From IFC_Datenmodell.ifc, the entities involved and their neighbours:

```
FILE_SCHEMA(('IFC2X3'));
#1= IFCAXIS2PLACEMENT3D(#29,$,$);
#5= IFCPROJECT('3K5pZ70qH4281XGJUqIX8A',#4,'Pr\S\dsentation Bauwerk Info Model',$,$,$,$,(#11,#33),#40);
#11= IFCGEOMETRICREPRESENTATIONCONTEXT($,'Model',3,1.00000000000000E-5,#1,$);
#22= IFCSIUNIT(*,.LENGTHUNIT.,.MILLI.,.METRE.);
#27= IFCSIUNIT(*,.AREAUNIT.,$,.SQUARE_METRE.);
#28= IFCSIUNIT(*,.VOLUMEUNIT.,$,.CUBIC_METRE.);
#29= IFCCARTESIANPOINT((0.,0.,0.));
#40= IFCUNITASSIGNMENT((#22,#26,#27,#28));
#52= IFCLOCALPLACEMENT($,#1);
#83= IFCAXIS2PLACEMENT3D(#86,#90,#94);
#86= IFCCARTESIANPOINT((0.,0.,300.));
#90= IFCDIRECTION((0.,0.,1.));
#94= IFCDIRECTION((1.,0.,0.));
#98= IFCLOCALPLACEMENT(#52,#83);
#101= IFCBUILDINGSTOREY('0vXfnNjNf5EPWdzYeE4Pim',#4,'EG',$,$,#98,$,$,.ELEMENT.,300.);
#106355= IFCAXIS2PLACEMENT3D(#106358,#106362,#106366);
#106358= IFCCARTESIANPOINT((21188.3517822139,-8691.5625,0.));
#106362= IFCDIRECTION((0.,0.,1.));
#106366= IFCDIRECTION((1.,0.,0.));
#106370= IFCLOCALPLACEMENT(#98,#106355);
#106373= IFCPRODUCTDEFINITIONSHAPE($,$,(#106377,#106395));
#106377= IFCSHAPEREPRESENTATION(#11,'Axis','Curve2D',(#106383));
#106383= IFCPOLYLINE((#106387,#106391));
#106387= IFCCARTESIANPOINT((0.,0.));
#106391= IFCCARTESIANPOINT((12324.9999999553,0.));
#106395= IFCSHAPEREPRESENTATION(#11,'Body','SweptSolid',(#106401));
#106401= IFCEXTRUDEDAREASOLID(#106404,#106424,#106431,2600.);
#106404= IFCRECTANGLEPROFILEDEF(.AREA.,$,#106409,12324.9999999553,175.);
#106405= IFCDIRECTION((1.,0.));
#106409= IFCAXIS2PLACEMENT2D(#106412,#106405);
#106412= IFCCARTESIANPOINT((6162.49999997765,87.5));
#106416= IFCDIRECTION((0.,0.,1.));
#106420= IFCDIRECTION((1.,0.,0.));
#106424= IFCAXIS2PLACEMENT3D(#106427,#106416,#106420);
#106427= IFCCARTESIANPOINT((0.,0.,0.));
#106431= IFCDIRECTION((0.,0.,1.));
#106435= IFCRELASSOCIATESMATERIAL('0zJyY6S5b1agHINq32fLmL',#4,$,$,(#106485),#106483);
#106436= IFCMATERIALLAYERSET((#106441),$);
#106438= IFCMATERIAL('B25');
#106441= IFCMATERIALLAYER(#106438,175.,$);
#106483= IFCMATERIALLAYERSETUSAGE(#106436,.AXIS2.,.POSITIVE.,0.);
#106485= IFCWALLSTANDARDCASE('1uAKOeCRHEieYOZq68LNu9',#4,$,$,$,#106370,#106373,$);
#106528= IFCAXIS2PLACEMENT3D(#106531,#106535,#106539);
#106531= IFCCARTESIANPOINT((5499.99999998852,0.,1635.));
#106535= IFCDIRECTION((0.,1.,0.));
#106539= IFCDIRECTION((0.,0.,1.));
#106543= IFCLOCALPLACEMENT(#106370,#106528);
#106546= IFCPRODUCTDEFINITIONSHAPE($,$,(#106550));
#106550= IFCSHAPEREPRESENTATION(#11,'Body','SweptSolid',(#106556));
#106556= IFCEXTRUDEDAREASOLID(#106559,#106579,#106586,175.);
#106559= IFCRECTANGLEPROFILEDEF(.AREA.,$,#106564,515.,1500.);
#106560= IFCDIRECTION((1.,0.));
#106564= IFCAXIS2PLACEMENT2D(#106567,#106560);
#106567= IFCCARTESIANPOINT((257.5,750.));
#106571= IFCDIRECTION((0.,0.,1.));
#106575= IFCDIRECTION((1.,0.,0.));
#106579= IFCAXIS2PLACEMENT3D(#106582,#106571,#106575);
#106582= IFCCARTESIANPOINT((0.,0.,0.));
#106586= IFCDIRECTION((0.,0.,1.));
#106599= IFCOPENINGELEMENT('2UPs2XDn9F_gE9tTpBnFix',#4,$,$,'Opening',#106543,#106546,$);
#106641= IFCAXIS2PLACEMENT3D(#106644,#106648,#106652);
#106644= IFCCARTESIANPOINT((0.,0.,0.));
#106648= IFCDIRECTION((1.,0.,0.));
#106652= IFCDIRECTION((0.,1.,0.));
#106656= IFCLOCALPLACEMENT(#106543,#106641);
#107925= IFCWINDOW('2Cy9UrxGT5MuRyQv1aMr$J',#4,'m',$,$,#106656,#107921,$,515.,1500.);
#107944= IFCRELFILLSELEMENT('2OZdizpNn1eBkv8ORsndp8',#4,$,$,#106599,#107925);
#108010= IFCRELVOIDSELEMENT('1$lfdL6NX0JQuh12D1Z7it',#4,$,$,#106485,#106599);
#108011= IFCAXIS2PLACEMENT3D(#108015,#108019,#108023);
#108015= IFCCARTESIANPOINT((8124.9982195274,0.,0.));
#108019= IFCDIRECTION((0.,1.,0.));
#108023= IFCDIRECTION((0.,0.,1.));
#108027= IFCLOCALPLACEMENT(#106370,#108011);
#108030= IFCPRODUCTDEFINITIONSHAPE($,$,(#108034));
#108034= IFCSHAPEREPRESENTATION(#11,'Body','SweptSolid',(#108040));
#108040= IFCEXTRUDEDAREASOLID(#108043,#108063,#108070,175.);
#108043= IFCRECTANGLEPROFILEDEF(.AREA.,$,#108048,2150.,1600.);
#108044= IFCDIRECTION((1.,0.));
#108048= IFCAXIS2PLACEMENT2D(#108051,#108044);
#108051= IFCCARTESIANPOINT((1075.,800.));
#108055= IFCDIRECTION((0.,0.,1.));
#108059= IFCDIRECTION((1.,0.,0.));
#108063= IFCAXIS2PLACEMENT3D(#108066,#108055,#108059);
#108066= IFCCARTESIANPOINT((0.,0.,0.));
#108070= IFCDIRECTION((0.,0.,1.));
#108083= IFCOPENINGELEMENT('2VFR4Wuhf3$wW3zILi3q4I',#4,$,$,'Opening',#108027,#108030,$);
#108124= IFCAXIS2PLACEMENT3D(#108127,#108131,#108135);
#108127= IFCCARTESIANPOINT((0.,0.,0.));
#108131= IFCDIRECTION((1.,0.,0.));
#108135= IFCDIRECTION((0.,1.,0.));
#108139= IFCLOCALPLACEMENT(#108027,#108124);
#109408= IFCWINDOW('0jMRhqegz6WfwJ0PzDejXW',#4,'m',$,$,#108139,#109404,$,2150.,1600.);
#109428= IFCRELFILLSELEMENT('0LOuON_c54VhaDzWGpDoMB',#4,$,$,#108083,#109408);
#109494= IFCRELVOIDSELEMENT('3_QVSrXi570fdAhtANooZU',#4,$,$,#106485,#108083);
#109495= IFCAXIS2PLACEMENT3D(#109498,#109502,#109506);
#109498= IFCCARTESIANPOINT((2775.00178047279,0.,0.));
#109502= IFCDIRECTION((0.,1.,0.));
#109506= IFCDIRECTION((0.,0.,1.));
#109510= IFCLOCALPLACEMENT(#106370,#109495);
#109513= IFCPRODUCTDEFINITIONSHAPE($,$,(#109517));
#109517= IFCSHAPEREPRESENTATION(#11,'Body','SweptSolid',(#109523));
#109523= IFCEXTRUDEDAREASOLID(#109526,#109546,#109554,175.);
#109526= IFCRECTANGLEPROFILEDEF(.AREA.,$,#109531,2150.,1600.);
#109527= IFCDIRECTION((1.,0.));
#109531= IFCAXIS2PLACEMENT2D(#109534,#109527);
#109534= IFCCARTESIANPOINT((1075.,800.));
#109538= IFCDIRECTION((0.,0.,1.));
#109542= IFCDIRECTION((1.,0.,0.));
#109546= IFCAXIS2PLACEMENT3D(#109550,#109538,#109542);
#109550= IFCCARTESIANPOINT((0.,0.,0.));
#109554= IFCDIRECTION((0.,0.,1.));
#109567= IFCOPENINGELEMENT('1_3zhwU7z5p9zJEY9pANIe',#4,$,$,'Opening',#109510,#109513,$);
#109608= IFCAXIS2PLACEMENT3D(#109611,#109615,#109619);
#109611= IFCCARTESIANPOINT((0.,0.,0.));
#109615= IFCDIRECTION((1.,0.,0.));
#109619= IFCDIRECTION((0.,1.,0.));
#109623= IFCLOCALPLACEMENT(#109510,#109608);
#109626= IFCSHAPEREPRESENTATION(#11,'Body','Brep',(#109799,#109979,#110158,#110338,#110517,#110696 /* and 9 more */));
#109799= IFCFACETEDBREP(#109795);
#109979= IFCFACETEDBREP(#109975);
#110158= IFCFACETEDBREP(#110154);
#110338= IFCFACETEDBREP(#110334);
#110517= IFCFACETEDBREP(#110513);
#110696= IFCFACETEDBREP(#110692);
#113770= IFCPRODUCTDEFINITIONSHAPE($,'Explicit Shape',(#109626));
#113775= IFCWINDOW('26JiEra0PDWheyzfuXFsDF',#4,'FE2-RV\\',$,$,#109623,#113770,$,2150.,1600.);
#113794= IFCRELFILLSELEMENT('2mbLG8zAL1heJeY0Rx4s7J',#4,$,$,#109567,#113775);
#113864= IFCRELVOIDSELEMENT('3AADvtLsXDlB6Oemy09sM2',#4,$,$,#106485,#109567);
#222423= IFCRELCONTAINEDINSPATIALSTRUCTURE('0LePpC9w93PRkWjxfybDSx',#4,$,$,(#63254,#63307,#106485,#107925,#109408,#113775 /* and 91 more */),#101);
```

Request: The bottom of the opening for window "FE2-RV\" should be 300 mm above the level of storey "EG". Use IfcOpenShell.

```python
import numpy as np
import ifcopenshell
import ifcopenshell.api.geometry
import ifcopenshell.geom
import ifcopenshell.util.element
import ifcopenshell.util.placement
import ifcopenshell.util.shape
import ifcopenshell.util.unit

model = ifcopenshell.open("IFC_Datenmodell.ifc")
unit_scale = ifcopenshell.util.unit.calculate_unit_scale(model)

window = model.by_guid("26JiEra0PDWheyzfuXFsDF")
opening = window.FillsVoids[0].RelatingOpeningElement
storey = ifcopenshell.util.element.get_container(window, ifc_class="IfcBuildingStorey")
level = ifcopenshell.util.placement.get_local_placement(storey.ObjectPlacement)[2, 3]

# The opening's origin need not be at the sill, so measure its lowest point.
shape = ifcopenshell.geom.create_shape(ifcopenshell.geom.settings(), opening)
bottom = ifcopenshell.util.shape.get_shape_bottom_elevation(shape, shape.geometry) / unit_scale
dz = level + 300.0 - bottom

shift = np.array([0.0, 0.0, dz])
# The window is placed relative to its opening, so it follows when the opening moves.
matrix = ifcopenshell.util.placement.get_local_placement(opening.ObjectPlacement)
matrix[:3, 3] += shift
ifcopenshell.api.geometry.edit_object_placement(
    model, product=opening, matrix=matrix, is_si=False, should_transform_children=True
)

print(f"moved by {dz * unit_scale:+.3f} m")

model.write("IFC_Datenmodell-out.ifc")
```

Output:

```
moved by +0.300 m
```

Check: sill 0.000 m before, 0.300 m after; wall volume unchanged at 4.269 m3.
